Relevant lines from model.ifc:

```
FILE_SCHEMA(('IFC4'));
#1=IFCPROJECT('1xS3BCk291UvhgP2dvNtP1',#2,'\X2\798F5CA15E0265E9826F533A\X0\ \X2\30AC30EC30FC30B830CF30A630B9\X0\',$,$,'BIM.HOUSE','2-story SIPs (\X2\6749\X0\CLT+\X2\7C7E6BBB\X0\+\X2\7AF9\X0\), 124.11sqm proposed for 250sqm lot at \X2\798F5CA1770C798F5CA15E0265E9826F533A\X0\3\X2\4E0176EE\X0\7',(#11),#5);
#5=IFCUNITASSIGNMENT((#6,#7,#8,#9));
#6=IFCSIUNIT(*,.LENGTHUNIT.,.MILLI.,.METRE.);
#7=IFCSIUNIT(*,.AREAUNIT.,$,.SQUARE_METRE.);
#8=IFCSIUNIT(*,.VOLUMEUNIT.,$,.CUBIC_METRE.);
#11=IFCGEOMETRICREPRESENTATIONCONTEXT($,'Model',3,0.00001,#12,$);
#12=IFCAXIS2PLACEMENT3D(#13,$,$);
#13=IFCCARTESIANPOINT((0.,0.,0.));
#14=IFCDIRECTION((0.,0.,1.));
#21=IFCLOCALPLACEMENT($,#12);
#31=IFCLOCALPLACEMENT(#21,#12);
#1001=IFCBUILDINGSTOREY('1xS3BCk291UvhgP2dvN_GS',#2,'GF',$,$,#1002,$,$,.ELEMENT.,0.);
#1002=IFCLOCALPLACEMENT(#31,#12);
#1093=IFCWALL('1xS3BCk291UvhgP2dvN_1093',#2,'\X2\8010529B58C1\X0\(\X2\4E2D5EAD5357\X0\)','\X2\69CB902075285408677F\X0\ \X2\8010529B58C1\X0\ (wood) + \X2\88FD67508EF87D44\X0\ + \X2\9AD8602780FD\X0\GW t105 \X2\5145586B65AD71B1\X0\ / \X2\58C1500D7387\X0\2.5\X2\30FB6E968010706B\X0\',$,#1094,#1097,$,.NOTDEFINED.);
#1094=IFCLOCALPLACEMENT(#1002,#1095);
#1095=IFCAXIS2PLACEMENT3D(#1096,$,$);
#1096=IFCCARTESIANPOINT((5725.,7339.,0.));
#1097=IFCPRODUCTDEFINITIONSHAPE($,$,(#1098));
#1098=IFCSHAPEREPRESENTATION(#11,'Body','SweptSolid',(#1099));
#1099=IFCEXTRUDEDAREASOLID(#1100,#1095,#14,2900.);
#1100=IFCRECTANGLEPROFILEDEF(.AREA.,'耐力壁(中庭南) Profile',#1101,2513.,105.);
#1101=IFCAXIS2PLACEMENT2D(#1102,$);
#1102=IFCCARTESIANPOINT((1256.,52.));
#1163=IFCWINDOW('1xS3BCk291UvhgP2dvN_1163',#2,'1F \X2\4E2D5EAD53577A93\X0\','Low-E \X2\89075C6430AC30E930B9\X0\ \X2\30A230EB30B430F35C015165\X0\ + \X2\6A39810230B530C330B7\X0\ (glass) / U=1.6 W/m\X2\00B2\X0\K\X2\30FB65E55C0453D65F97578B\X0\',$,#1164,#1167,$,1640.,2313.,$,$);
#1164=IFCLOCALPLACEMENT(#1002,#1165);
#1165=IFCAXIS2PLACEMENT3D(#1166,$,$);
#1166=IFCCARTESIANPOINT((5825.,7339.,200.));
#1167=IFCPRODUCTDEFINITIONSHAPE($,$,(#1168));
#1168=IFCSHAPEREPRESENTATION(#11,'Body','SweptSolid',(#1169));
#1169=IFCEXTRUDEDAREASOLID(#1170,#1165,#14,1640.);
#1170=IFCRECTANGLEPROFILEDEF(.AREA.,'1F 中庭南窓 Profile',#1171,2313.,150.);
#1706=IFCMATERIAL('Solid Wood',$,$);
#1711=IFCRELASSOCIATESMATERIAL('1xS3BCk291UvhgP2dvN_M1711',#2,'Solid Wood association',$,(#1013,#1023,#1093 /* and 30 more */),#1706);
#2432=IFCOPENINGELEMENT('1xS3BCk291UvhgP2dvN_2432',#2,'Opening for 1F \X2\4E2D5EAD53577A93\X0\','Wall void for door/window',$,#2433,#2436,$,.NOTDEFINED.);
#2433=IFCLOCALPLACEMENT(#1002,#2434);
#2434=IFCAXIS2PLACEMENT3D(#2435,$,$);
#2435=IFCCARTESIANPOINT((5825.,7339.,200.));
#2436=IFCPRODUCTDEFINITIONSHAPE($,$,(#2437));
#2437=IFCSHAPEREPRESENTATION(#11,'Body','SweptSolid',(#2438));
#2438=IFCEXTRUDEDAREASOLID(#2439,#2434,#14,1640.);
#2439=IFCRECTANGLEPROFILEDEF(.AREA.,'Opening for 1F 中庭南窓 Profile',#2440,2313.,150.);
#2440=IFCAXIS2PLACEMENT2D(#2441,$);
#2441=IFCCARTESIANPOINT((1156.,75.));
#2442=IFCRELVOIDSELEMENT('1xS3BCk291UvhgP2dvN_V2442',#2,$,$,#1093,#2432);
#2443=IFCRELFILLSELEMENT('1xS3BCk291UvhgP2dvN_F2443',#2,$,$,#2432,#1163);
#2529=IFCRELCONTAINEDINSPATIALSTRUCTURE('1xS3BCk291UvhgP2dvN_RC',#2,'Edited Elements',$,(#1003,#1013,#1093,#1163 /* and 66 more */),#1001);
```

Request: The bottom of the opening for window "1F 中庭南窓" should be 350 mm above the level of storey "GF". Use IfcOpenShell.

```python
import numpy as np
import ifcopenshell
import ifcopenshell.api.geometry
import ifcopenshell.geom
import ifcopenshell.util.element
import ifcopenshell.util.placement
import ifcopenshell.util.shape
import ifcopenshell.util.unit

model = ifcopenshell.open("model.ifc")
unit_scale = ifcopenshell.util.unit.calculate_unit_scale(model)

window = model.by_guid("1xS3BCk291UvhgP2dvN_1163")
opening = window.FillsVoids[0].RelatingOpeningElement
storey = ifcopenshell.util.element.get_container(window, ifc_class="IfcBuildingStorey")
level = ifcopenshell.util.placement.get_local_placement(storey.ObjectPlacement)[2, 3]

# The opening's origin need not be at the sill, so measure its lowest point.
shape = ifcopenshell.geom.create_shape(ifcopenshell.geom.settings(), opening)
bottom = ifcopenshell.util.shape.get_shape_bottom_elevation(shape, shape.geometry) / unit_scale
dz = level + 350.0 - bottom

shift = np.array([0.0, 0.0, dz])
# The window is not placed relative to its opening, so move both.
for product in (opening, window):
    matrix = ifcopenshell.util.placement.get_local_placement(product.ObjectPlacement)
    matrix[:3, 3] += shift
    ifcopenshell.api.geometry.edit_object_placement(model, product=product, matrix=matrix, is_si=False)

print(f"moved by {dz * unit_scale:+.3f} m")

model.write("model_updated.ifc")
```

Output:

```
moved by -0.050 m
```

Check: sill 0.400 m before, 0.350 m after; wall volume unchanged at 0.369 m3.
